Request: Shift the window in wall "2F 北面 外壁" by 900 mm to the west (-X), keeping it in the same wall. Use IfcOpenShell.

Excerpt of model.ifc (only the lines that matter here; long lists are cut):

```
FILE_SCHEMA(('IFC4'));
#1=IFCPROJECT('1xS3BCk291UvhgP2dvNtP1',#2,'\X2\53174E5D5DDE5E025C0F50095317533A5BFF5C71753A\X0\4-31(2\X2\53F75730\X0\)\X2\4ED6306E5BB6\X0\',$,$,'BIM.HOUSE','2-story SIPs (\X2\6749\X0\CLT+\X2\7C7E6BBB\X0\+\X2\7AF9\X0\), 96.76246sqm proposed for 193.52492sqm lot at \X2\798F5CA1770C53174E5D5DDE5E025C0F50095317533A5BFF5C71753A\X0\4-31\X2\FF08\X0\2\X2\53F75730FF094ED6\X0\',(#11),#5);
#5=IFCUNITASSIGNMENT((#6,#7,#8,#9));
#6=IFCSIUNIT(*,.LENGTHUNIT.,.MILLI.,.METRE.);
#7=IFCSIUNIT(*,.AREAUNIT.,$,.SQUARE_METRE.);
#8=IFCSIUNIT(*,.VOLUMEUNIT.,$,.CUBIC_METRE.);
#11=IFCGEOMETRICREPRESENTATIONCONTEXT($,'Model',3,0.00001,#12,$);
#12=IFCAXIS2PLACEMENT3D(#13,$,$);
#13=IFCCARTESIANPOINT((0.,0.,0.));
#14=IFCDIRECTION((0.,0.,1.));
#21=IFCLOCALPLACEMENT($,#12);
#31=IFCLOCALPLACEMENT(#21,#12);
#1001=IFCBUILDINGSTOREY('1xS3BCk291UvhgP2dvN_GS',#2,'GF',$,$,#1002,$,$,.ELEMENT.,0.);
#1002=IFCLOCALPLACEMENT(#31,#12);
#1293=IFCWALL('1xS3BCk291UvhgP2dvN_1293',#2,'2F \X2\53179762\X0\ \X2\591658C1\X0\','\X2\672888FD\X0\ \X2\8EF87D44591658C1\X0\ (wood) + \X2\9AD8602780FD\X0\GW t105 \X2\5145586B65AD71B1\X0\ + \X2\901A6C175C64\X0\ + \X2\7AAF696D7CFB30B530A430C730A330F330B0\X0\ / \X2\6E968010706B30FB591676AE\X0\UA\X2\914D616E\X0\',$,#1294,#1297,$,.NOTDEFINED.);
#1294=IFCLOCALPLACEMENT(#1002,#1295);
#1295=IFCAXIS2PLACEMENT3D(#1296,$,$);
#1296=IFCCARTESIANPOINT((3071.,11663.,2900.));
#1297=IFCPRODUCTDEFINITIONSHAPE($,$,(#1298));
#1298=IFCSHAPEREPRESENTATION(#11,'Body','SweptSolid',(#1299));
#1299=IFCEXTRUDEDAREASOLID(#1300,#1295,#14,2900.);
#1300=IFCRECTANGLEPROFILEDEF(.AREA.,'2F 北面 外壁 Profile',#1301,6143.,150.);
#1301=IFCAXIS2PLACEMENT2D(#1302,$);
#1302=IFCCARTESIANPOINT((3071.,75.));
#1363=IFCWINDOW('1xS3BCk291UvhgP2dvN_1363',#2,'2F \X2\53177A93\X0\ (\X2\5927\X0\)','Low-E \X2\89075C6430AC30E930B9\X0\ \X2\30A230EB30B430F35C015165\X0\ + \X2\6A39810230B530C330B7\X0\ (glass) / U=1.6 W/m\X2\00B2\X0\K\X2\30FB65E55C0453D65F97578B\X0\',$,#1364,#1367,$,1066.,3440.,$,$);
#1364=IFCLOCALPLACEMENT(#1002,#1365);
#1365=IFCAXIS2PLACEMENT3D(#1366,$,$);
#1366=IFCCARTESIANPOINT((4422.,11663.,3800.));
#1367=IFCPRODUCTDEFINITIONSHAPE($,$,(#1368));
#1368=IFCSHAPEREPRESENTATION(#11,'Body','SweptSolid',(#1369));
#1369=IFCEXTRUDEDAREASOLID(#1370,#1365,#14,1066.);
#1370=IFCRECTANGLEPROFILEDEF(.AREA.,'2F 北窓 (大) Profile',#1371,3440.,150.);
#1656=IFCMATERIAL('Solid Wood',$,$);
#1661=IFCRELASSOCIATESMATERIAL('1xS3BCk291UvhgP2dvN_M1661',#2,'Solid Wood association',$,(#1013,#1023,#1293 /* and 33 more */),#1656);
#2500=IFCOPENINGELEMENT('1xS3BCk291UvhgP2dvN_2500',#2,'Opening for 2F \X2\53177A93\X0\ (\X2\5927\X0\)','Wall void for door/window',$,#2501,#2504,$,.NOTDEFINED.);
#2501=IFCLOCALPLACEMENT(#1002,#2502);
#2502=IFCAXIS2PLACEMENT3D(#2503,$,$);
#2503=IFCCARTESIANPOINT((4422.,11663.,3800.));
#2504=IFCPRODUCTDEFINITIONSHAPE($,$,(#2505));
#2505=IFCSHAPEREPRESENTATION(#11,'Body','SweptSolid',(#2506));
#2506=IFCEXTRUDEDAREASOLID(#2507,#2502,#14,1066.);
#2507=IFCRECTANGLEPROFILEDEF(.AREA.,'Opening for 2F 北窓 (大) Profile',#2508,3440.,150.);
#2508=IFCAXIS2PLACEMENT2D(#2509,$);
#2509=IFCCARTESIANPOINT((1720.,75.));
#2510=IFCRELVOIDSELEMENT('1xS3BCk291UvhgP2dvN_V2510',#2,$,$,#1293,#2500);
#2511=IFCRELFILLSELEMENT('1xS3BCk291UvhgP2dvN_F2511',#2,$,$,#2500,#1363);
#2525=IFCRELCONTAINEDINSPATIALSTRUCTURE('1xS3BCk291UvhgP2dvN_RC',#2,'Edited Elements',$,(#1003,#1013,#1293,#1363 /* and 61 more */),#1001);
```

```python
import ifcopenshell
import ifcopenshell.api.geometry
import ifcopenshell.util.placement

model = ifcopenshell.open("model.ifc")

window = model.by_guid("1xS3BCk291UvhgP2dvN_1363")
opening = window.FillsVoids[0].RelatingOpeningElement
wall = opening.VoidsElements[0].RelatingBuildingElement

wall_matrix = ifcopenshell.util.placement.get_local_placement(wall.ObjectPlacement)
shift = wall_matrix[:3, 0] * -900.0
before = ifcopenshell.util.placement.get_local_placement(window.ObjectPlacement)[:3, 3].copy()

# The window is not placed relative to its opening, so move both.
for product in (opening, window):
    matrix = ifcopenshell.util.placement.get_local_placement(product.ObjectPlacement)
    matrix[:3, 3] += shift
    ifcopenshell.api.geometry.edit_object_placement(model, product=product, matrix=matrix, is_si=False)

after = ifcopenshell.util.placement.get_local_placement(window.ObjectPlacement)[:3, 3]
print("window moved by", (after - before).round(3) + 0.0)

model.write("model_rev.ifc")
```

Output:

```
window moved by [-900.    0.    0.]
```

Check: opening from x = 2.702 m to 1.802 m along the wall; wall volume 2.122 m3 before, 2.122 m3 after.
